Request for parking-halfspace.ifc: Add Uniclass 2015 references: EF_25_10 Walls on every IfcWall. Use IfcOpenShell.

First a look at what the model holds.

```python
import ifcopenshell

model = ifcopenshell.open("parking-halfspace.ifc")
print(model.schema)
print("classifications:", [c.Name for c in model.by_type("IfcClassification")])
for ifc_class in ("IfcDoor", "IfcRoof", "IfcStair", "IfcWall", "IfcWindow"):
    print(ifc_class, len(model.by_type(ifc_class)))
```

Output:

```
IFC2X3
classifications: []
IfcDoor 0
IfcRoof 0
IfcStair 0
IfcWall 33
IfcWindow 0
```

```python
import ifcopenshell
import ifcopenshell.api.classification

model = ifcopenshell.open("parking-halfspace.ifc")

# IFC2X3 requires Source and Edition and has no link from the project to the system.
system = model.create_entity("IfcClassification", Source="NBS", Edition="2015", Name="Uniclass 2015")

codes = {
    "IfcWall": ("EF_25_10", "Walls"),
}
for ifc_class, (code, name) in codes.items():
    products = model.by_type(ifc_class)
    ifcopenshell.api.classification.add_reference(
        model, products=products, classification=system, identification=code, name=name
    )
    print(code, len(products))

model.write("parking-halfspace_rev.ifc")
```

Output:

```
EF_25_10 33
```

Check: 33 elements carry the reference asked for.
